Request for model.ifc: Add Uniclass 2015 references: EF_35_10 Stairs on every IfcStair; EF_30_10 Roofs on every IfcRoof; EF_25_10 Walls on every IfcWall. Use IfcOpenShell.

First a look at what the model holds.

```python
import ifcopenshell

model = ifcopenshell.open("model.ifc")
print(model.schema)
print("classifications:", [c.Name for c in model.by_type("IfcClassification")])
for ifc_class in ("IfcDoor", "IfcRoof", "IfcStair", "IfcWall", "IfcWindow"):
    print(ifc_class, len(model.by_type(ifc_class)))
```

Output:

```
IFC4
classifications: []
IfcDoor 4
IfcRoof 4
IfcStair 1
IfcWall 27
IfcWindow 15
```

```python
import ifcopenshell
import ifcopenshell.api.classification

model = ifcopenshell.open("model.ifc")

system = ifcopenshell.api.classification.add_classification(model, classification="Uniclass 2015")

codes = {
    "IfcStair": ("EF_35_10", "Stairs"),
    "IfcRoof": ("EF_30_10", "Roofs"),
    "IfcWall": ("EF_25_10", "Walls"),
}
for ifc_class, (code, name) in codes.items():
    products = model.by_type(ifc_class)
    ifcopenshell.api.classification.add_reference(
        model, products=products, classification=system, identification=code, name=name
    )
    print(code, len(products))

model.write("model-out.ifc")
```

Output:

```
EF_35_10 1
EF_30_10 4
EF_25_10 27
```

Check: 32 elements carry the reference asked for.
